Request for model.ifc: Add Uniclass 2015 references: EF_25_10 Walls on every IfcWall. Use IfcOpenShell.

First a look at what the model holds.

```python
import ifcopenshell

model = ifcopenshell.open("model.ifc")
print(model.schema)
print("classifications:", [c.Name for c in model.by_type("IfcClassification")])
for ifc_class in ("IfcDoor", "IfcRoof", "IfcStair", "IfcWall", "IfcWindow"):
    print(ifc_class, len(model.by_type(ifc_class)))
```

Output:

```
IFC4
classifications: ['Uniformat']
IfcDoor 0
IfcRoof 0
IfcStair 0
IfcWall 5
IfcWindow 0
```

```python
import ifcopenshell
import ifcopenshell.api.classification

model = ifcopenshell.open("model.ifc")

system = ifcopenshell.api.classification.add_classification(model, classification="Uniclass 2015")

codes = {
    "IfcWall": ("EF_25_10", "Walls"),
}
for ifc_class, (code, name) in codes.items():
    products = model.by_type(ifc_class)
    ifcopenshell.api.classification.add_reference(
        model, products=products, classification=system, identification=code, name=name
    )
    print(code, len(products))

model.write("model_updated.ifc")
```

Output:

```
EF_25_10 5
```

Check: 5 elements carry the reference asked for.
